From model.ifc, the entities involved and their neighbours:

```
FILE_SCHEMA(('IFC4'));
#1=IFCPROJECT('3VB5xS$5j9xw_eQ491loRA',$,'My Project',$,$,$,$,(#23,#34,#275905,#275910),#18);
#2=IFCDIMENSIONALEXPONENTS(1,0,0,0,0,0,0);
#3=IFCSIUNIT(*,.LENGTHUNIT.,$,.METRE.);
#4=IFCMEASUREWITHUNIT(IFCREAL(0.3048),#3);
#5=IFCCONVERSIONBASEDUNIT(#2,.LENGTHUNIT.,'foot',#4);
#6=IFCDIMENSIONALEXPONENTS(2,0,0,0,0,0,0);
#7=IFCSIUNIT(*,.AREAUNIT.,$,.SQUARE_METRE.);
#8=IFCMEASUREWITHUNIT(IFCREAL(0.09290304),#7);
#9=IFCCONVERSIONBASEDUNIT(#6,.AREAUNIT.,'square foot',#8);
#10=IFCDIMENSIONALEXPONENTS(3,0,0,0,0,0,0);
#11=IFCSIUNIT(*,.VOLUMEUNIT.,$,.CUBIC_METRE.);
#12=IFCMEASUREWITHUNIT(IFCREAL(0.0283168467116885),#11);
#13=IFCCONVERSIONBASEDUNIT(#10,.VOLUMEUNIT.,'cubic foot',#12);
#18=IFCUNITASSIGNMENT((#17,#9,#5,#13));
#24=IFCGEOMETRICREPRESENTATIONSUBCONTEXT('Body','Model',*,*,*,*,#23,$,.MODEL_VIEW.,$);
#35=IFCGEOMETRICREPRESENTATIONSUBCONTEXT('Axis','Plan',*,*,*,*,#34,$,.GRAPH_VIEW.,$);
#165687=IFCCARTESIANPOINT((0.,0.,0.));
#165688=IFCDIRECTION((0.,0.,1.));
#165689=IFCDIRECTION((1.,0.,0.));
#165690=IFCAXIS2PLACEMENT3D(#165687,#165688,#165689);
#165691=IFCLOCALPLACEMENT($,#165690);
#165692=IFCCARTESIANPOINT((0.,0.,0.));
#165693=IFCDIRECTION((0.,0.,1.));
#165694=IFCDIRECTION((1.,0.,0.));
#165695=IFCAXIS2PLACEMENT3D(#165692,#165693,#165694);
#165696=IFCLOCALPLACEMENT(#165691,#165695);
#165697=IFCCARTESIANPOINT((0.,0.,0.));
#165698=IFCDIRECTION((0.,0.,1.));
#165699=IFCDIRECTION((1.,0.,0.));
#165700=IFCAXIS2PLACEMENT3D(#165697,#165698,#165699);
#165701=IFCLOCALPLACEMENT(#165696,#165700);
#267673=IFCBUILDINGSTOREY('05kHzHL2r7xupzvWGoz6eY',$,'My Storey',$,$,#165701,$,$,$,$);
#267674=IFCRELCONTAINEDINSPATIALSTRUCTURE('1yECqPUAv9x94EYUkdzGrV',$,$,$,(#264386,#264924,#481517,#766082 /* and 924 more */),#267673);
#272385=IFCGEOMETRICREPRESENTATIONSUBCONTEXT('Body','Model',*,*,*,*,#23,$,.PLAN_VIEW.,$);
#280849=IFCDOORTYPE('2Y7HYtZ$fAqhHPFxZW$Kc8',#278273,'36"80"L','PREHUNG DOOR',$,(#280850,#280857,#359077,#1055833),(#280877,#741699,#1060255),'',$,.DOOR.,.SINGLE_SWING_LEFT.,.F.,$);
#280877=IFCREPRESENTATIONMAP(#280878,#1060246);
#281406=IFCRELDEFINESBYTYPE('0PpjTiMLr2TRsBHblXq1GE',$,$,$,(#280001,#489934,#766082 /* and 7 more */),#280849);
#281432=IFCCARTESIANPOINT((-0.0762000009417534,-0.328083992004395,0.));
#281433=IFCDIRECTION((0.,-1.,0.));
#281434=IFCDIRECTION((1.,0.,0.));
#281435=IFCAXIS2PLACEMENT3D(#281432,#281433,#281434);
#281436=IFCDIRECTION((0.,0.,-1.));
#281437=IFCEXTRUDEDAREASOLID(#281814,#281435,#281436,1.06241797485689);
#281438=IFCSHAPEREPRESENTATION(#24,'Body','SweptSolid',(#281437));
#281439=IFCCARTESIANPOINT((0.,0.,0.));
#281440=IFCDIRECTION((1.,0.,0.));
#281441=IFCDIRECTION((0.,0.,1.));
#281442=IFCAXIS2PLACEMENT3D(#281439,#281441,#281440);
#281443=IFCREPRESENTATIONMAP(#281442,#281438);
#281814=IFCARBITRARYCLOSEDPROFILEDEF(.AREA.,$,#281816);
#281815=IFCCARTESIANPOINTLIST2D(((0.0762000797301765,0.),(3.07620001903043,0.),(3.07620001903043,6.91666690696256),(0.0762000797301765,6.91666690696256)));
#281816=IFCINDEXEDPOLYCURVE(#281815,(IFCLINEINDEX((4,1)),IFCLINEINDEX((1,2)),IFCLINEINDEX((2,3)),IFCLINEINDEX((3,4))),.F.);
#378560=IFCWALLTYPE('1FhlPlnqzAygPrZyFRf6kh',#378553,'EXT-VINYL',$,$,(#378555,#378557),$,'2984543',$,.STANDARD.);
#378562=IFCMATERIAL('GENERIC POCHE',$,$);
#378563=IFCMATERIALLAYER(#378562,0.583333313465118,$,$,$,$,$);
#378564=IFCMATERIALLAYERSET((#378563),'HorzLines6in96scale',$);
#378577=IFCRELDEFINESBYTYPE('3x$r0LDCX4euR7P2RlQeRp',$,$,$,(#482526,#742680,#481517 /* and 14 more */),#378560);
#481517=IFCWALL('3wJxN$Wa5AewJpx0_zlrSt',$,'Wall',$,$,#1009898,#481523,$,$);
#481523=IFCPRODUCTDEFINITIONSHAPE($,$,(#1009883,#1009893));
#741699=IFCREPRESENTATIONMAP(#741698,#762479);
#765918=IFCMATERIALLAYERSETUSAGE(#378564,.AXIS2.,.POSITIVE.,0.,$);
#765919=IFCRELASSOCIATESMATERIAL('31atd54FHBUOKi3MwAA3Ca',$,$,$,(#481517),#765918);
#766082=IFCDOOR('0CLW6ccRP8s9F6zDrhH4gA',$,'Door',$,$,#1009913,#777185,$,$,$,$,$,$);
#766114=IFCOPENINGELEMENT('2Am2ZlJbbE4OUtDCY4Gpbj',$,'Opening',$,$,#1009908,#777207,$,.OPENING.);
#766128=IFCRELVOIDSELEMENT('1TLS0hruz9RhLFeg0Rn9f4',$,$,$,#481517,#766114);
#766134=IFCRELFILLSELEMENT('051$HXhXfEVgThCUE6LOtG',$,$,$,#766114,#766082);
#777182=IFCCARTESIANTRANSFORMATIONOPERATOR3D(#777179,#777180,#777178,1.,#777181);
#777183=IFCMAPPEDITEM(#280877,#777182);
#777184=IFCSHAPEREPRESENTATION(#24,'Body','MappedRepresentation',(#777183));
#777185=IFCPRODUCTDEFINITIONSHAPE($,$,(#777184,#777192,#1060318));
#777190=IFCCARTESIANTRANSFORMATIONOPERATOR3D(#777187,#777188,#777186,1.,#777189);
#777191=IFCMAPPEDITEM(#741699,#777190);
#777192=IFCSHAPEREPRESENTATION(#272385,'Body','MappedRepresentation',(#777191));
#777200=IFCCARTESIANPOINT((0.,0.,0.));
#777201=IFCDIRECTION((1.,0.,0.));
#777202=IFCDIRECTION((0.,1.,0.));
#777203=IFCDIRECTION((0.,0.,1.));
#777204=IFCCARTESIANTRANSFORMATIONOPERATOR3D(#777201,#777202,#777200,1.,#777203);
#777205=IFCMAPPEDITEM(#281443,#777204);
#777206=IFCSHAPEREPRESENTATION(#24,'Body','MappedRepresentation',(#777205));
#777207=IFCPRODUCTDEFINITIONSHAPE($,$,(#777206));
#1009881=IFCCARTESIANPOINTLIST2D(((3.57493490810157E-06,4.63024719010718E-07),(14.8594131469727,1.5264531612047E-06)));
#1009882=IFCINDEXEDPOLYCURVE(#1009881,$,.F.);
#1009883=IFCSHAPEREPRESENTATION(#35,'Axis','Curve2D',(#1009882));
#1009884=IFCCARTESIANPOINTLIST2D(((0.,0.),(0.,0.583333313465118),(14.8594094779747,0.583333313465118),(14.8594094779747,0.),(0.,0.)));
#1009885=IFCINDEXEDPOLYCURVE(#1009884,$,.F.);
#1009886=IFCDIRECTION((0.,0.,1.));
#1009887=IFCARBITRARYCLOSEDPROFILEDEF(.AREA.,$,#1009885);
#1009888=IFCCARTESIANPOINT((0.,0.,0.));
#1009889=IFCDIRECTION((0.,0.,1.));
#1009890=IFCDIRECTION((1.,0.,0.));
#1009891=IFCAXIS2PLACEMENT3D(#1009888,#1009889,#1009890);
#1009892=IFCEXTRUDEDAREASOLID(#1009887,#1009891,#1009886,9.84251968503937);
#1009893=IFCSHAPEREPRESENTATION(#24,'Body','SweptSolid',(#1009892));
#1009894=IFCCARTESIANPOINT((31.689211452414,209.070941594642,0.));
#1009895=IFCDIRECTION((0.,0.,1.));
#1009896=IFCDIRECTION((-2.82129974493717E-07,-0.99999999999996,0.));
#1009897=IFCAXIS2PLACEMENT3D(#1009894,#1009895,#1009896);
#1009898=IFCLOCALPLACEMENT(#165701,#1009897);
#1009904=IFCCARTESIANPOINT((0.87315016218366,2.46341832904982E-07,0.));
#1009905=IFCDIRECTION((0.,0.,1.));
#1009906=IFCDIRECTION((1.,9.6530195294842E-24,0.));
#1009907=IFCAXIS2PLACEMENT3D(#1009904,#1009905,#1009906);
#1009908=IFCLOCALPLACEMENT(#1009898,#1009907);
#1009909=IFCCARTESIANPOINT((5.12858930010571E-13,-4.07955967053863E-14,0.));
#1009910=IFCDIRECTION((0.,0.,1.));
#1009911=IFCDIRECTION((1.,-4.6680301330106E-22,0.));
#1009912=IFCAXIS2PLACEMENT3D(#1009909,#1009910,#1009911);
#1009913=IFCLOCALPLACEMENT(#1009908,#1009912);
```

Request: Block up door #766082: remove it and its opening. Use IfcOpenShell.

```python
import ifcopenshell
import ifcopenshell.api.feature
import ifcopenshell.api.root
import ifcopenshell.geom
import ifcopenshell.util.shape

model = ifcopenshell.open("model.ifc")
settings = ifcopenshell.geom.settings()


def volume(element):
    """Net volume in cubic metres, openings subtracted."""
    shape = ifcopenshell.geom.create_shape(settings, element)
    return ifcopenshell.util.shape.get_volume(shape.geometry)


door = model.by_guid("0CLW6ccRP8s9F6zDrhH4gA")
opening = door.FillsVoids[0].RelatingOpeningElement
wall = opening.VoidsElements[0].RelatingBuildingElement
before = volume(wall)

ifcopenshell.api.root.remove_product(model, product=door)
ifcopenshell.api.feature.remove_feature(model, feature=opening)

after = volume(wall)

print(f"wall volume {before:.3f} -> {after:.3f} m3")

model.write("model_edited.ifc")
```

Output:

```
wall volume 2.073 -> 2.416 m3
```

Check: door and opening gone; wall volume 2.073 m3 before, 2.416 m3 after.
